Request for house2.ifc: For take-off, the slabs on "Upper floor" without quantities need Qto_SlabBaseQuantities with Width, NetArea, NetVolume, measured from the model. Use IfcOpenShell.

First a look at what the model holds.

```python
import ifcopenshell
import ifcopenshell.util.element
import ifcopenshell.util.unit

model = ifcopenshell.open("house2.ifc")
print(model.schema)
for unit_type in ("LENGTHUNIT", "AREAUNIT", "VOLUMEUNIT"):
    print(unit_type, ifcopenshell.util.unit.calculate_unit_scale(model, unit_type))
storey = next(s for s in model.by_type("IfcBuildingStorey") if s.Name == "Upper floor")
slabs = [e for e in ifcopenshell.util.element.get_decomposition(storey) if e.is_a("IfcSlab")]
for e in sorted(slabs, key=lambda e: e.id()):
    print(e.id(), e.is_a(), e.Name, list(ifcopenshell.util.element.get_psets(e, qtos_only=True)), sep=" | ")
```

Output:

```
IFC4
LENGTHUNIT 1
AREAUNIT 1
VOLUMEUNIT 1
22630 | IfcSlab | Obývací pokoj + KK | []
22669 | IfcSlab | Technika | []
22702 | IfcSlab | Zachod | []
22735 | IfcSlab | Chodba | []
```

```python
import ifcopenshell
import ifcopenshell.api.pset
import ifcopenshell.geom
import ifcopenshell.util.element
import ifcopenshell.util.shape
import ifcopenshell.util.unit

model = ifcopenshell.open("house2.ifc")
unit_scale = ifcopenshell.util.unit.calculate_unit_scale(model)
area_scale = ifcopenshell.util.unit.calculate_unit_scale(model, "AREAUNIT")
volume_scale = ifcopenshell.util.unit.calculate_unit_scale(model, "VOLUMEUNIT")
settings = ifcopenshell.geom.settings()

storey = next(s for s in model.by_type("IfcBuildingStorey") if s.Name == "Upper floor")
slabs = [e for e in ifcopenshell.util.element.get_decomposition(storey) if e.is_a("IfcSlab")]

for e in sorted(slabs, key=lambda e: e.id()):
    if ifcopenshell.util.element.get_psets(e, qtos_only=True, should_inherit=False):
        continue
    # Geometry comes back in metres, in the element's own axes.
    shape = ifcopenshell.geom.create_shape(settings, e)
    values = {
        "Width": ifcopenshell.util.shape.get_z(shape.geometry) / unit_scale,
        "NetArea": ifcopenshell.util.shape.get_footprint_area(shape.geometry) / area_scale,
        "NetVolume": ifcopenshell.util.shape.get_volume(shape.geometry) / volume_scale,
    }
    qto = ifcopenshell.api.pset.add_qto(model, product=e, name="Qto_SlabBaseQuantities")
    ifcopenshell.api.pset.edit_qto(model, qto=qto, properties=values)
    print(e.id(), {k: round(v, 3) for k, v in values.items()})

model.write("house2_updated.ifc")
```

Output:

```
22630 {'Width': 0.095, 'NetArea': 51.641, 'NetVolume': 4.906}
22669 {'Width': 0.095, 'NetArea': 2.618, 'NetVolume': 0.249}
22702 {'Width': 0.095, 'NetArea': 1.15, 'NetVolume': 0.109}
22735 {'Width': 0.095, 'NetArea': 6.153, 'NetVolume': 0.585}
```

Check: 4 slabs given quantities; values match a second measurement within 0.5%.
